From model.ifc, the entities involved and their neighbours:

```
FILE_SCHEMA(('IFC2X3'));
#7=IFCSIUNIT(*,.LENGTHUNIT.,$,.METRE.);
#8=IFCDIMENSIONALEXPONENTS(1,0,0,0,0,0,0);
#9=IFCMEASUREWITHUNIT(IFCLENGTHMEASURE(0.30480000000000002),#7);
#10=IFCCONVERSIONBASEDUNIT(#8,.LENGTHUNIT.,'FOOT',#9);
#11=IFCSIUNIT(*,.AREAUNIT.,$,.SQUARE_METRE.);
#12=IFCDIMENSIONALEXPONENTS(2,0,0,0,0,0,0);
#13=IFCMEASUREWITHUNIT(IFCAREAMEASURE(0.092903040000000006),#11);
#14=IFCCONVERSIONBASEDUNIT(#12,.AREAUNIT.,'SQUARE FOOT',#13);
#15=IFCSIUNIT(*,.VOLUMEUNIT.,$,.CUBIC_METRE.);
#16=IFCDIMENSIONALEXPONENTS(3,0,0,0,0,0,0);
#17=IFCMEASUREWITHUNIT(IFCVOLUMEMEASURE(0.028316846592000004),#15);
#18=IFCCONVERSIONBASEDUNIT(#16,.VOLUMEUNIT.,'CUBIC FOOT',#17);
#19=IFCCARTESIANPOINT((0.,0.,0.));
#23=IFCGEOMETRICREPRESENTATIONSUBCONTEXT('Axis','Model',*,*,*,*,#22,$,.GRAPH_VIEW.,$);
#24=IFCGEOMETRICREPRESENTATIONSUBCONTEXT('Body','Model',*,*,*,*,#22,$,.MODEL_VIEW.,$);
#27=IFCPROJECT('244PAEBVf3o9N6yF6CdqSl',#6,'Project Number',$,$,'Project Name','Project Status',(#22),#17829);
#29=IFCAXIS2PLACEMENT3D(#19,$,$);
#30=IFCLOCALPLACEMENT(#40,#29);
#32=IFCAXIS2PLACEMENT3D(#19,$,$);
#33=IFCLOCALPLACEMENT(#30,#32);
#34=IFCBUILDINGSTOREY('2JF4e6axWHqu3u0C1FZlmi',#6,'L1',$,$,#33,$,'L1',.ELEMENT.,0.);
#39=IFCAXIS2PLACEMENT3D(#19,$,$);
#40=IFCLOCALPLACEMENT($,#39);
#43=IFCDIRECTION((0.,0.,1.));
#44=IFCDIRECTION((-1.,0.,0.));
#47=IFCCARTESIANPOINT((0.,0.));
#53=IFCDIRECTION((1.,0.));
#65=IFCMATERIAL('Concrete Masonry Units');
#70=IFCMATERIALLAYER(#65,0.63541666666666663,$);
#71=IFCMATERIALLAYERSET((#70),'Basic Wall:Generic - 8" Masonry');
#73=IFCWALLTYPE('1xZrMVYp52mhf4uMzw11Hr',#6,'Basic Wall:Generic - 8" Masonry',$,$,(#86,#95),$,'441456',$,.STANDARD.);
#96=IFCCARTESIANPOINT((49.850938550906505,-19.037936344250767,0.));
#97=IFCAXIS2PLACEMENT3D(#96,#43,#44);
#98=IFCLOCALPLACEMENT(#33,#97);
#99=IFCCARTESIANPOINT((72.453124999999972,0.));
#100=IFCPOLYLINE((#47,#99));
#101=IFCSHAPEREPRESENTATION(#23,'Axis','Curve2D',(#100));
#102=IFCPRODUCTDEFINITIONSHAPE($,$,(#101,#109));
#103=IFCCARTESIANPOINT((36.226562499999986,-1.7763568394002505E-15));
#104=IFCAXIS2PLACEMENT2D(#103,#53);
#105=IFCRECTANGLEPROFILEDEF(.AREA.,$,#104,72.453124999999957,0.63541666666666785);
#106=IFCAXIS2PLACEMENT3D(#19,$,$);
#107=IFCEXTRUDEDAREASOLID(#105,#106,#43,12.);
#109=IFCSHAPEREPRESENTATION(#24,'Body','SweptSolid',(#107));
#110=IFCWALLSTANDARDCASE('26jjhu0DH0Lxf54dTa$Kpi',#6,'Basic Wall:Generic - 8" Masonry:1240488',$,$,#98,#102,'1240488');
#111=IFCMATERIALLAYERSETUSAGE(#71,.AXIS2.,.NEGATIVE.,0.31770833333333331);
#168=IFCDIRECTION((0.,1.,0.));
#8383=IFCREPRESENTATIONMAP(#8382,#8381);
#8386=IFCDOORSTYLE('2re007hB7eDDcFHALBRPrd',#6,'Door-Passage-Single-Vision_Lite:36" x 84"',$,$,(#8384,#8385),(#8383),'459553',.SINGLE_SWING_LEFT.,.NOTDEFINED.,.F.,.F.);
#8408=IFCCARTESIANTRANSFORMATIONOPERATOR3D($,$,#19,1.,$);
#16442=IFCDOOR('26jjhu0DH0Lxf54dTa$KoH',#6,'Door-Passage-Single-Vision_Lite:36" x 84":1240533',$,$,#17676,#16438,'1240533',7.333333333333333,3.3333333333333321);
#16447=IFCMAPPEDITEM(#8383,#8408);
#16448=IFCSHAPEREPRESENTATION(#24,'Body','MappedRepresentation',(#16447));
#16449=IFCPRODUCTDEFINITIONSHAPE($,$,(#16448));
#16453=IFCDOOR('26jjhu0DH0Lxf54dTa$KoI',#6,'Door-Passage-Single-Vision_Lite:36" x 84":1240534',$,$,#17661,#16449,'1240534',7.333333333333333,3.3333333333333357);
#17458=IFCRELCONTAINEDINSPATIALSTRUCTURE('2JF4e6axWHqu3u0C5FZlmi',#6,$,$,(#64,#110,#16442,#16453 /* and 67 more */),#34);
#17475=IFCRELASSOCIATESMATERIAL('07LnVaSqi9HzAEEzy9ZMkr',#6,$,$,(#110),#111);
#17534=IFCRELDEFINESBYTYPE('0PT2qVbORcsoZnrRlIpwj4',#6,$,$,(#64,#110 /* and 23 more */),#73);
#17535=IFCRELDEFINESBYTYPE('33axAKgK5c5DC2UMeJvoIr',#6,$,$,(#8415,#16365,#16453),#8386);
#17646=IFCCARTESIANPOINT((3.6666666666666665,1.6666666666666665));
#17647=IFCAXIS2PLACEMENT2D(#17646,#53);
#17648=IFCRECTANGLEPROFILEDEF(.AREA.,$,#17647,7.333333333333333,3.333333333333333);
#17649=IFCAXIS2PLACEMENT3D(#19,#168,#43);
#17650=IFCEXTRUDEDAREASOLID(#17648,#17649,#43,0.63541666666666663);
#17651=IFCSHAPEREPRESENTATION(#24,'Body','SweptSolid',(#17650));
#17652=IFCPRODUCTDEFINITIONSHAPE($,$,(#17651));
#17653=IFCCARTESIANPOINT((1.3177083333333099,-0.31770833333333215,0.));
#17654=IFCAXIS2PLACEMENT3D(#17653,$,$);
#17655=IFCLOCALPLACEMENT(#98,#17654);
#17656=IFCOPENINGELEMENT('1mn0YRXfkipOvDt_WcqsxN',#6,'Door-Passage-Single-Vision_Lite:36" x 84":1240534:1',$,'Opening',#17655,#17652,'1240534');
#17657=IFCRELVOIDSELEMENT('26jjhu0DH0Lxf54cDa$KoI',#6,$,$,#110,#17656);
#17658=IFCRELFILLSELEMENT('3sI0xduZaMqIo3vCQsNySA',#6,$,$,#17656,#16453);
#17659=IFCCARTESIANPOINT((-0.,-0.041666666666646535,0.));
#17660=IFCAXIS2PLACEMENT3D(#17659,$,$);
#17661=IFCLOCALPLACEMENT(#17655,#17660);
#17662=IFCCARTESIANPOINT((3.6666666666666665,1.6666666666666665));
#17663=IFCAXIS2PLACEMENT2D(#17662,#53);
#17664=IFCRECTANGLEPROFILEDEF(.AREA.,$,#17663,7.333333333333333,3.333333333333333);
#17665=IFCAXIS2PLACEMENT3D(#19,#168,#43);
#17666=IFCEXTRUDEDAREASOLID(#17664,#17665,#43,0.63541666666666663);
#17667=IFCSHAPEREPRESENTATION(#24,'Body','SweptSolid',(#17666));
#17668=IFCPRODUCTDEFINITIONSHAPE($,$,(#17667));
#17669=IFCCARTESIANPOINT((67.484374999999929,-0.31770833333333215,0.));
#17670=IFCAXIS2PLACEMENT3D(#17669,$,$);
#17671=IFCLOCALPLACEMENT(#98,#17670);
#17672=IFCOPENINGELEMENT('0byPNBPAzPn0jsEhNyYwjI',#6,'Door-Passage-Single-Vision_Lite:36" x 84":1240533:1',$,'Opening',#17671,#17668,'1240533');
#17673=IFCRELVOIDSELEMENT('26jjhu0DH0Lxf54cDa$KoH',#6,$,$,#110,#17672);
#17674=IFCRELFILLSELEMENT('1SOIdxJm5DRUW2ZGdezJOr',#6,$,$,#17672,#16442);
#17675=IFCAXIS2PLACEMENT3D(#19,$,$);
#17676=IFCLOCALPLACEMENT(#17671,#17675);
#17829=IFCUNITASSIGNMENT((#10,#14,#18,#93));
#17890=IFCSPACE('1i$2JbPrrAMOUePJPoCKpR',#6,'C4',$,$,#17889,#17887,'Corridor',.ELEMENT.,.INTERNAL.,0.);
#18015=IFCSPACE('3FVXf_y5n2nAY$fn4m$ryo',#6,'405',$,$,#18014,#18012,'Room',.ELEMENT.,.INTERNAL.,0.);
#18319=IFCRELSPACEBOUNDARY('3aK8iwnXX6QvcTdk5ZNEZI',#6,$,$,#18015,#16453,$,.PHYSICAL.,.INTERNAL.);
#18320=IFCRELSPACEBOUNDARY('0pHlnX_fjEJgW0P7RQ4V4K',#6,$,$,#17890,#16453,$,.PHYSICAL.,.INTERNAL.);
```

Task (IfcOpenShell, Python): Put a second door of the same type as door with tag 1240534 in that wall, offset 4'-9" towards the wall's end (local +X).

```python
import ifcopenshell
import ifcopenshell.api.feature
import ifcopenshell.api.geometry
import ifcopenshell.api.root
import ifcopenshell.geom
import ifcopenshell.util.element
import ifcopenshell.util.placement
import ifcopenshell.util.shape
import ifcopenshell.util.unit

model = ifcopenshell.open("model.ifc")
unit_scale = ifcopenshell.util.unit.calculate_unit_scale(model)
settings = ifcopenshell.geom.settings()


def volume(element):
    """Net volume in cubic metres, openings subtracted."""
    shape = ifcopenshell.geom.create_shape(settings, element)
    return ifcopenshell.util.shape.get_volume(shape.geometry)


def reuse_history(source, copy):
    """copy_class also copies each property set's owner history, people and application; keep the originals."""
    for rel in copy.IsDefinedBy:
        if rel.is_a("IfcRelDefinesByProperties") and (history := rel.RelatingPropertyDefinition.OwnerHistory):
            rel.RelatingPropertyDefinition.OwnerHistory = source.OwnerHistory
            ifcopenshell.util.element.remove_deep2(model, history)


door = model.by_guid("26jjhu0DH0Lxf54dTa$KoI")
opening = door.FillsVoids[0].RelatingOpeningElement
wall = opening.VoidsElements[0].RelatingBuildingElement
before = volume(wall)
shift = ifcopenshell.util.placement.get_local_placement(wall.ObjectPlacement)[:3, 0] * 57 * 0.0254 / unit_scale

# copy_class copies the void relationship, type, container and properties, but no geometry.
new_opening = ifcopenshell.api.root.copy_class(model, product=opening)
new_opening.Representation = ifcopenshell.util.element.copy_deep(
    model, opening.Representation, exclude=["IfcGeometricRepresentationContext", "IfcRepresentationMap"]
)
new_opening.Name = 'Door-Passage-Single-Vision_Lite:36" x 84"'
new_opening.Tag = None
new_door = ifcopenshell.api.root.copy_class(model, product=door)
new_door.Representation = ifcopenshell.util.element.copy_deep(
    model, door.Representation, exclude=["IfcGeometricRepresentationContext", "IfcRepresentationMap"]
)
new_door.Name = 'Door-Passage-Single-Vision_Lite:36" x 84"'
new_door.Tag = None
reuse_history(door, new_door)
fills = ifcopenshell.api.feature.add_filling(model, opening=new_opening, element=new_door)
fills.OwnerHistory = new_door.OwnerHistory  # required in IFC2X3

for old, new in ((opening, new_opening), (door, new_door)):
    matrix = ifcopenshell.util.placement.get_local_placement(old.ObjectPlacement)
    matrix[:3, 3] += shift
    ifcopenshell.api.geometry.edit_object_placement(model, product=new, matrix=matrix, is_si=False)

after = volume(wall)

print(f"wall volume {before:.3f} -> {after:.3f} m3")

model.write("model_rev.ifc")
```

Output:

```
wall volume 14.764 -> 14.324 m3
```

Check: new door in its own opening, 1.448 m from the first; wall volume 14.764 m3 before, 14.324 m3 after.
